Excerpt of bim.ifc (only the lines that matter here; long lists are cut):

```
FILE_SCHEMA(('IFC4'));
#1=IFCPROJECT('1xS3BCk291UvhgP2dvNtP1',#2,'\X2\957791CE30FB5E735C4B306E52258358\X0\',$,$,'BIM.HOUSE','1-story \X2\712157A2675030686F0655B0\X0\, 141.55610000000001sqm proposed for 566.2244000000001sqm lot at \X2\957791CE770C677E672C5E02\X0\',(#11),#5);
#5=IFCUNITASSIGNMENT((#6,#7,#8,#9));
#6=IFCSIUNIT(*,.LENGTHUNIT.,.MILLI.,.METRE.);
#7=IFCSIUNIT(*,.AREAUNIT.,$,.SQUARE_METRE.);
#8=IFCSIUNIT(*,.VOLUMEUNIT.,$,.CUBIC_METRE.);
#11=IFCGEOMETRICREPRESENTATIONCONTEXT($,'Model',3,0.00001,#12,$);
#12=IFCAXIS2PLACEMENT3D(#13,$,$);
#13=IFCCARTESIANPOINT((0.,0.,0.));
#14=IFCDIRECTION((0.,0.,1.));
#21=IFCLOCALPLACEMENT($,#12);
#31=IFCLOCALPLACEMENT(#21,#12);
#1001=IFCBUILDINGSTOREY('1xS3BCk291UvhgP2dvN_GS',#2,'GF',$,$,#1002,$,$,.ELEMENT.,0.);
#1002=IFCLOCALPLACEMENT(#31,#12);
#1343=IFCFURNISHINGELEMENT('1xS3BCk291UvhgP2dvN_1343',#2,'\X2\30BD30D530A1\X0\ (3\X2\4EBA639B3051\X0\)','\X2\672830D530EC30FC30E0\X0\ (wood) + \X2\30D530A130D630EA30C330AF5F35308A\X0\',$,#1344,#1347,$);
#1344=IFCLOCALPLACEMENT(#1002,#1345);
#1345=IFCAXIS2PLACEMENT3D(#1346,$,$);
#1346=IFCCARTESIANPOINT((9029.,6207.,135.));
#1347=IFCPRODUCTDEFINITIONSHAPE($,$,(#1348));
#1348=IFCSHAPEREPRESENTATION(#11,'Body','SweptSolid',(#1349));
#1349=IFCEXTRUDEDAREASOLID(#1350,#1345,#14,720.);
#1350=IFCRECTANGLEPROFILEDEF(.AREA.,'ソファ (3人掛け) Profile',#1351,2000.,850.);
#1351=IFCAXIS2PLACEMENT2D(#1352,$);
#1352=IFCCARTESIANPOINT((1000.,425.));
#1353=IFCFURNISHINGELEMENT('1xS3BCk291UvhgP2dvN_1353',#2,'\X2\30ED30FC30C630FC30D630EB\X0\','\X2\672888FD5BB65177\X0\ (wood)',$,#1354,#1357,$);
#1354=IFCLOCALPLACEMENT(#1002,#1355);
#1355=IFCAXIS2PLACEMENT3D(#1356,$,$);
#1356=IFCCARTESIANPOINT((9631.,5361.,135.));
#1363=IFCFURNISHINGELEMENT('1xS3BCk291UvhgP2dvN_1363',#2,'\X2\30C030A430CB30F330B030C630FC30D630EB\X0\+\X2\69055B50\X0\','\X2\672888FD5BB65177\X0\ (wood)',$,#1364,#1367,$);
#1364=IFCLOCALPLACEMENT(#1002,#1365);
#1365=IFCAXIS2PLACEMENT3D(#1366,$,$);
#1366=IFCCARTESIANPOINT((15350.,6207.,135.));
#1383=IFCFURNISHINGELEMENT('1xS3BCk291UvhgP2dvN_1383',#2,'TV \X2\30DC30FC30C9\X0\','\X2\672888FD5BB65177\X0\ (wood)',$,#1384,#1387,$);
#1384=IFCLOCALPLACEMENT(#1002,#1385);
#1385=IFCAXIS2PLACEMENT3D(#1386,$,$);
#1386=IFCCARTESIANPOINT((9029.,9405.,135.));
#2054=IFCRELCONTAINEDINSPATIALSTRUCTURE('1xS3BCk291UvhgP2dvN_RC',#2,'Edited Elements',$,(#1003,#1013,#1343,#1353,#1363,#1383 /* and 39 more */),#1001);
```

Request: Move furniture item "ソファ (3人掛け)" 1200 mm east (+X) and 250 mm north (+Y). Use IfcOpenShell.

```python
import ifcopenshell
import ifcopenshell.api.geometry
import ifcopenshell.util.placement
import ifcopenshell.util.unit

model = ifcopenshell.open("bim.ifc")
unit_scale = ifcopenshell.util.unit.calculate_unit_scale(model)

item = model.by_guid("1xS3BCk291UvhgP2dvN_1343")
matrix = ifcopenshell.util.placement.get_local_placement(item.ObjectPlacement)
matrix[0, 3] += 1.2 / unit_scale
matrix[1, 3] += 0.25 / unit_scale
ifcopenshell.api.geometry.edit_object_placement(model, product=item, matrix=matrix, is_si=False)

print(ifcopenshell.util.placement.get_local_placement(item.ObjectPlacement).round(3) + 0.0)

model.write("bim_v2.ifc")
```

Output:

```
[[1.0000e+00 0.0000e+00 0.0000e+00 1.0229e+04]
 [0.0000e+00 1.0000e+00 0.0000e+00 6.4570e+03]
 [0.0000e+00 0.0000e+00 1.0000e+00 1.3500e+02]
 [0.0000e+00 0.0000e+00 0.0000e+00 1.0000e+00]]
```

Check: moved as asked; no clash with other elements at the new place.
